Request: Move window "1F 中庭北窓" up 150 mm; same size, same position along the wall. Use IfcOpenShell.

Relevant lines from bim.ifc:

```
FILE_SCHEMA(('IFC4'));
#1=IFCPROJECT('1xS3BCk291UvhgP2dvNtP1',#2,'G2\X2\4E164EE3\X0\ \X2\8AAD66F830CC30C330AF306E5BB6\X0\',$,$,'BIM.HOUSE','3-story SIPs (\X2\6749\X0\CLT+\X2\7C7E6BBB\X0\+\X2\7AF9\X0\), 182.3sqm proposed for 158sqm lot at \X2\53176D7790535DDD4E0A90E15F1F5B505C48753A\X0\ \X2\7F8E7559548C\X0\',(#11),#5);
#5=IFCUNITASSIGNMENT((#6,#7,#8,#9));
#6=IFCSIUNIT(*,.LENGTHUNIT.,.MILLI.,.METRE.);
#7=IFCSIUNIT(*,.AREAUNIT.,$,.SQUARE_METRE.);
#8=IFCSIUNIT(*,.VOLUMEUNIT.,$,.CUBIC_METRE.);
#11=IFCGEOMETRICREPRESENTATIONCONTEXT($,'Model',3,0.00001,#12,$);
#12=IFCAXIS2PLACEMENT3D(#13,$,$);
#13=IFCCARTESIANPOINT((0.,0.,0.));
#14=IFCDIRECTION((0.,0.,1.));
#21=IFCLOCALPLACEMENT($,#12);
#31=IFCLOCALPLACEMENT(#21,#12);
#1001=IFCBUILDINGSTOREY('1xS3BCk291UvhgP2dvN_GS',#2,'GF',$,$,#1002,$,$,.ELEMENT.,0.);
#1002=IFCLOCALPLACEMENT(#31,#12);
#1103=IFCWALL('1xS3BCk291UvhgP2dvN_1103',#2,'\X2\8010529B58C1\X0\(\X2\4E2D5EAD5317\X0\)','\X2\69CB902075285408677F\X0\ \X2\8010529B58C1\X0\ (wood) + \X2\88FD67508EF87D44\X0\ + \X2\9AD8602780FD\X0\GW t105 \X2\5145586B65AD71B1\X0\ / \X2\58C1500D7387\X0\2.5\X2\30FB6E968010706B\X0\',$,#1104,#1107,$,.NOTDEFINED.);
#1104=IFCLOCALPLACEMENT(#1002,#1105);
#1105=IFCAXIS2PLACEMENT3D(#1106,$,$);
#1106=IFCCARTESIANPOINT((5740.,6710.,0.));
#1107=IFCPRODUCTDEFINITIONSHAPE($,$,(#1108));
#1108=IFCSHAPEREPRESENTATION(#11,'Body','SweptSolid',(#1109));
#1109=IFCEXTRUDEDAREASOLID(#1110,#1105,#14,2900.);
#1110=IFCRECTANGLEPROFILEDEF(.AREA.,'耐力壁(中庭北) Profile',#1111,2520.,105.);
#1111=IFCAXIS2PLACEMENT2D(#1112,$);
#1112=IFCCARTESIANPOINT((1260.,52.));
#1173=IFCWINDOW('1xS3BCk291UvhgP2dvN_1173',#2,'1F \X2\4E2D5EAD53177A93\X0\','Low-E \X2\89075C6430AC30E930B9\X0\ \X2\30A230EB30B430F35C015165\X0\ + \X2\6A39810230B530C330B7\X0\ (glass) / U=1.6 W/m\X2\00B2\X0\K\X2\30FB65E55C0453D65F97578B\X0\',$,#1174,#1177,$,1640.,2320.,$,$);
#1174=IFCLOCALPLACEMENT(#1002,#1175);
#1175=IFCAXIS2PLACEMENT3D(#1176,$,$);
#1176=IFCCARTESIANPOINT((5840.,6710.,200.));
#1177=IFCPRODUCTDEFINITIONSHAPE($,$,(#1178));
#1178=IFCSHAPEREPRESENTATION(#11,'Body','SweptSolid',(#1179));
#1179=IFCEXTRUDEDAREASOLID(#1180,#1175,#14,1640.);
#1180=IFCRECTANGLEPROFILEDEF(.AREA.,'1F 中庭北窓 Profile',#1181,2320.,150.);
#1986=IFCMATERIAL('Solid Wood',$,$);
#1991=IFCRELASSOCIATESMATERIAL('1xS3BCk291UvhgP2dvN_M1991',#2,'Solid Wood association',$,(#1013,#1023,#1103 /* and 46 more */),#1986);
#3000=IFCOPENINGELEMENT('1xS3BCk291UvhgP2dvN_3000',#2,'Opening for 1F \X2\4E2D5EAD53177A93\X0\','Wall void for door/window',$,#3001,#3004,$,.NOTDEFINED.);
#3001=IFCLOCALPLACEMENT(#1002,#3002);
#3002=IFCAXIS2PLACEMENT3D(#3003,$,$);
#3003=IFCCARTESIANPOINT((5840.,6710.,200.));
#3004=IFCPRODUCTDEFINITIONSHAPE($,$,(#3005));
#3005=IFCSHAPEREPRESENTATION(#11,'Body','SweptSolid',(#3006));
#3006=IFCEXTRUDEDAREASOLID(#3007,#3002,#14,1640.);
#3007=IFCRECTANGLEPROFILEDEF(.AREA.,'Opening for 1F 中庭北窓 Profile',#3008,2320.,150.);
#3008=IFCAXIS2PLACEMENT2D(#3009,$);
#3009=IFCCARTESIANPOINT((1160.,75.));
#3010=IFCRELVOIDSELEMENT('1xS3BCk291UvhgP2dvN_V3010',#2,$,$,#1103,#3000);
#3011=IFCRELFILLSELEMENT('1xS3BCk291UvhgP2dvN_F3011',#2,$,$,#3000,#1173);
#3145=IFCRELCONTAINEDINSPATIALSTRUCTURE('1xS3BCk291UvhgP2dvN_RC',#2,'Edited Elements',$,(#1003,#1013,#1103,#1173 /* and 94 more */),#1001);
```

```python
import numpy as np
import ifcopenshell
import ifcopenshell.api.geometry
import ifcopenshell.util.placement
import ifcopenshell.util.unit

model = ifcopenshell.open("bim.ifc")
unit_scale = ifcopenshell.util.unit.calculate_unit_scale(model)

window = model.by_guid("1xS3BCk291UvhgP2dvN_1173")
opening = window.FillsVoids[0].RelatingOpeningElement
dz = 150.0

shift = np.array([0.0, 0.0, dz])
# The window is not placed relative to its opening, so move both.
for product in (opening, window):
    matrix = ifcopenshell.util.placement.get_local_placement(product.ObjectPlacement)
    matrix[:3, 3] += shift
    ifcopenshell.api.geometry.edit_object_placement(model, product=product, matrix=matrix, is_si=False)

print(f"moved by {dz * unit_scale:+.3f} m")

model.write("bim_v2.ifc")
```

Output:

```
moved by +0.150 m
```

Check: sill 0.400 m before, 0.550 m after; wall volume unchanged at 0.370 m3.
